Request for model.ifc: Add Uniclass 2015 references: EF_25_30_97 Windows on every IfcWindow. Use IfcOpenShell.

First a look at what the model holds.

```python
import ifcopenshell

model = ifcopenshell.open("model.ifc")
print(model.schema)
print("classifications:", [c.Name for c in model.by_type("IfcClassification")])
for ifc_class in ("IfcDoor", "IfcRoof", "IfcStair", "IfcWall", "IfcWindow"):
    print(ifc_class, len(model.by_type(ifc_class)))
```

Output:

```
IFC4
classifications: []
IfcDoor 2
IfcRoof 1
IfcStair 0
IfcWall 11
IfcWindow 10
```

```python
import ifcopenshell
import ifcopenshell.api.classification

model = ifcopenshell.open("model.ifc")

system = ifcopenshell.api.classification.add_classification(model, classification="Uniclass 2015")

codes = {
    "IfcWindow": ("EF_25_30_97", "Windows"),
}
for ifc_class, (code, name) in codes.items():
    products = model.by_type(ifc_class)
    ifcopenshell.api.classification.add_reference(
        model, products=products, classification=system, identification=code, name=name
    )
    print(code, len(products))

model.write("model-out.ifc")
```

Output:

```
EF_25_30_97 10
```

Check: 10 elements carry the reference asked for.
